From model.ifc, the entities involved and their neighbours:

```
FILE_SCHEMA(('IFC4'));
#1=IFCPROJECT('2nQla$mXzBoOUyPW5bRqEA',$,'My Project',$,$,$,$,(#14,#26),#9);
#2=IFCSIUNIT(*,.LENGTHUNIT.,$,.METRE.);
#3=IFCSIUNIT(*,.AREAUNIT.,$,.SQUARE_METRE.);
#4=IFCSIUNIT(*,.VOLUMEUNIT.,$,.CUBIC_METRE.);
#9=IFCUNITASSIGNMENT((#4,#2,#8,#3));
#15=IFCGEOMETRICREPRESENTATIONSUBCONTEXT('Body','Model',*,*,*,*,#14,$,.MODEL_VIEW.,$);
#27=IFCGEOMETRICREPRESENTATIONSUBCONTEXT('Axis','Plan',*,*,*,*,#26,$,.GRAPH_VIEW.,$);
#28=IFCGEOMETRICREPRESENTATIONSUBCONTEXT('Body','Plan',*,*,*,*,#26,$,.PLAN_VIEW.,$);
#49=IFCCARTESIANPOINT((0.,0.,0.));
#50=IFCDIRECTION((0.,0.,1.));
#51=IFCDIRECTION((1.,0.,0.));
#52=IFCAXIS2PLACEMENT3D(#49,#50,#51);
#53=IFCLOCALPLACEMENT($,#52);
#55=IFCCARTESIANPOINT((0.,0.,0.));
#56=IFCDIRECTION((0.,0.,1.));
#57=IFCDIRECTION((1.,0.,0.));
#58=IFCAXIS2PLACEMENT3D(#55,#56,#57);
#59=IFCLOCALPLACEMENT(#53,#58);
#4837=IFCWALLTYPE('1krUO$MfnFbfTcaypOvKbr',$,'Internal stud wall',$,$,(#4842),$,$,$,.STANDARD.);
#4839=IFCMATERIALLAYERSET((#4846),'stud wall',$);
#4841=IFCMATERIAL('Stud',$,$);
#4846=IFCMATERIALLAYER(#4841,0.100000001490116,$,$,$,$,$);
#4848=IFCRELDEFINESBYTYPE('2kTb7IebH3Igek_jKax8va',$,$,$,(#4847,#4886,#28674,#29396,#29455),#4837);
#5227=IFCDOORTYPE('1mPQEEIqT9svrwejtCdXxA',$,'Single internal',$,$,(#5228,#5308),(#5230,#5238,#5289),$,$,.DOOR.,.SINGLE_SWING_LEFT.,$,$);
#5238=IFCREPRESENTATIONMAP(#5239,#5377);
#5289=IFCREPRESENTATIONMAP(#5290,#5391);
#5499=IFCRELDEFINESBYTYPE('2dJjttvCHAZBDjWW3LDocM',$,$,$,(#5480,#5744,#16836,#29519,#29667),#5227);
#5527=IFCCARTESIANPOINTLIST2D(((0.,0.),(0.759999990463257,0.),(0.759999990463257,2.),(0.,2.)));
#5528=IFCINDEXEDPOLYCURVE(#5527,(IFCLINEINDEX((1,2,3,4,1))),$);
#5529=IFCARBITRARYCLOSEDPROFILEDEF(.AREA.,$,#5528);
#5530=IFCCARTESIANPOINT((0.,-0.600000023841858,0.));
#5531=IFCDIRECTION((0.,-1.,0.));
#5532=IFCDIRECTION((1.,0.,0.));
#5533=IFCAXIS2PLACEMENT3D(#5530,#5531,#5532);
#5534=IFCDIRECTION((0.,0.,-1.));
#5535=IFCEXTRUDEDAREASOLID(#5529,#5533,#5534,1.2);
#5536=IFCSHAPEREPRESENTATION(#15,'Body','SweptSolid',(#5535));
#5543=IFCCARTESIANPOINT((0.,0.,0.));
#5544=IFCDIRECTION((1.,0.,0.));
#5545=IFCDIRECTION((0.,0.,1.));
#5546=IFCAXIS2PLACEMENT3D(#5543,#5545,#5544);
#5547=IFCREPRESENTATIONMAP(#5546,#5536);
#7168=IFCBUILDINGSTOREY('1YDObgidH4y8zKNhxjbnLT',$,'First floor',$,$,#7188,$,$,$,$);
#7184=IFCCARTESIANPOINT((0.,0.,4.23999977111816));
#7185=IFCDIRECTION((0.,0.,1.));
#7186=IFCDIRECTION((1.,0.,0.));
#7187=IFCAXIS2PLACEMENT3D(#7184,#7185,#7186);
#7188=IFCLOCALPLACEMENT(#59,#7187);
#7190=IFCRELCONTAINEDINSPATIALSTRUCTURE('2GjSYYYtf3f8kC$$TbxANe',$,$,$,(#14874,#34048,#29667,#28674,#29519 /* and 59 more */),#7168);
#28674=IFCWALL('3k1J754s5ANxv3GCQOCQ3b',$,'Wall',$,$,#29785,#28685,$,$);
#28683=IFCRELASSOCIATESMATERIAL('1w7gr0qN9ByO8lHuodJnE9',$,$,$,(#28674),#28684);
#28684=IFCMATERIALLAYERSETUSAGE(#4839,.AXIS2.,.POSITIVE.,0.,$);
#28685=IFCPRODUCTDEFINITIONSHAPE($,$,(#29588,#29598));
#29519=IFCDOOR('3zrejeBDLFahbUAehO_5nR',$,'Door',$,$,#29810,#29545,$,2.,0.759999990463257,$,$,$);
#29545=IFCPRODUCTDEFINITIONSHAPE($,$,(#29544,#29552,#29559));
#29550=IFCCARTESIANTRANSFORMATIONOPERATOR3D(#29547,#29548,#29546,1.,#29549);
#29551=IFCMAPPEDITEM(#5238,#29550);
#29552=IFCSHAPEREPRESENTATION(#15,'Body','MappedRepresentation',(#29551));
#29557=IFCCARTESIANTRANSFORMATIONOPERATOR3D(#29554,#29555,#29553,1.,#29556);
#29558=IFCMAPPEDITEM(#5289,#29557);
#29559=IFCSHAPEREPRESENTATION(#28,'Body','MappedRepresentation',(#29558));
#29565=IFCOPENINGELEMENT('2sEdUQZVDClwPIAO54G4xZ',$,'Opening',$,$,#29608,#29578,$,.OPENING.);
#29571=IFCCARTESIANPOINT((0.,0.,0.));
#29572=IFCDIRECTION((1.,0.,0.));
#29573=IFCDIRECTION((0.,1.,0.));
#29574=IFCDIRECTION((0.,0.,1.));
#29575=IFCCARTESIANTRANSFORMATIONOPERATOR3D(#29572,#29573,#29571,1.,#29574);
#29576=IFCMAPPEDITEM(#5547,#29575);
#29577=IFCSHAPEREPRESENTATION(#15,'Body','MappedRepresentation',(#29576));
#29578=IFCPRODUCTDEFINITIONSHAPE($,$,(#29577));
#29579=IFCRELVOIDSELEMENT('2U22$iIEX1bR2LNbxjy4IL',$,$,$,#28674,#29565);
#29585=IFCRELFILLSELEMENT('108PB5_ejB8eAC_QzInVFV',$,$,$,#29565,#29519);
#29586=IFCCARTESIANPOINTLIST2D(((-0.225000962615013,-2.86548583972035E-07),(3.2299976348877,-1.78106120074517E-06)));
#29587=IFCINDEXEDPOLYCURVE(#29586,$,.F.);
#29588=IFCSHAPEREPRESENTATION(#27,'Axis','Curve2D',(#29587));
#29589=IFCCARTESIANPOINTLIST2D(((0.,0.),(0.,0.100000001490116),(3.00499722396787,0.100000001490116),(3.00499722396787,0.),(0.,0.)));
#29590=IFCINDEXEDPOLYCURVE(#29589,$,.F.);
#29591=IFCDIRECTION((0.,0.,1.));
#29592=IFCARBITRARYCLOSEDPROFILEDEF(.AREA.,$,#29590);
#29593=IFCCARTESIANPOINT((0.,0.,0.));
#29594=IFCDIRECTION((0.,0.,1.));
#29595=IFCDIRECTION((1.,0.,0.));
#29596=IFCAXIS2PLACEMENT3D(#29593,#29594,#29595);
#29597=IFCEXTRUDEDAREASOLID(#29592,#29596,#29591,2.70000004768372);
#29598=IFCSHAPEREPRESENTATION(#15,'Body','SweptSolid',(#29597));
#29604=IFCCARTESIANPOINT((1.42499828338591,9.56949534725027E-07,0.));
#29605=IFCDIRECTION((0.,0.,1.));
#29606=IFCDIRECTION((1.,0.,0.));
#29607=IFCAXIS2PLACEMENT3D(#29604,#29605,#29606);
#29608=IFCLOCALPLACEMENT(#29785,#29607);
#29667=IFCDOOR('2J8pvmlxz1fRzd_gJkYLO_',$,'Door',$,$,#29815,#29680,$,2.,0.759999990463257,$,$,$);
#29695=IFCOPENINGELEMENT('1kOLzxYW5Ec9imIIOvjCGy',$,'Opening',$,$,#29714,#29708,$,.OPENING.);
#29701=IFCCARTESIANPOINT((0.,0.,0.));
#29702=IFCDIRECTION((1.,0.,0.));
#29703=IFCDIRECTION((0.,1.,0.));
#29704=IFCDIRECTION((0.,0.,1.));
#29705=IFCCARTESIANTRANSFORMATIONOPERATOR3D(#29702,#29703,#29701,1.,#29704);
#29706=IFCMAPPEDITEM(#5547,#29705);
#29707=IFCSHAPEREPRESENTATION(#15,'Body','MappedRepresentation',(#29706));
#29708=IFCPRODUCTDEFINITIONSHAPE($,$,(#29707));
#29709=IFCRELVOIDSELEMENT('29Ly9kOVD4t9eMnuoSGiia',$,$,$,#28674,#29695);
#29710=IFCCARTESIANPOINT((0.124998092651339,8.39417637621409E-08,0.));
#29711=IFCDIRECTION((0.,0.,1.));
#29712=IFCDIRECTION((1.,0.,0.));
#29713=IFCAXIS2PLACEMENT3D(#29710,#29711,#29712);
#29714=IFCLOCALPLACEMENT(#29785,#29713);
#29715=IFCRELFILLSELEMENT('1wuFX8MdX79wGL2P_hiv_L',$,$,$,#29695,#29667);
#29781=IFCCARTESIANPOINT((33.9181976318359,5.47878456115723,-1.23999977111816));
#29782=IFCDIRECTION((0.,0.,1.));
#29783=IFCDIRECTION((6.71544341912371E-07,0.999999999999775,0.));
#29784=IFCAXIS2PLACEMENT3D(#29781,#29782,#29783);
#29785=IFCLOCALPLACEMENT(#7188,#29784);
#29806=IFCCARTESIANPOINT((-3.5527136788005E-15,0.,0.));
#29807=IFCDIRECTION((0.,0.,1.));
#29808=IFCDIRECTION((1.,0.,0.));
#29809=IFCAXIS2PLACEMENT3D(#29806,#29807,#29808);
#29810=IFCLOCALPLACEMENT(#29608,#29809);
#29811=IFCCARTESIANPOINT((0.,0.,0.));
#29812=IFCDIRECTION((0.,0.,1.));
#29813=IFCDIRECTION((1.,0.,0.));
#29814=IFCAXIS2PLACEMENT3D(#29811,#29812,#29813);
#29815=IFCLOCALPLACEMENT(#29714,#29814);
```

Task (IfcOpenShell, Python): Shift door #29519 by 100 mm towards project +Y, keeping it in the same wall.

```python
import ifcopenshell
import ifcopenshell.api.geometry
import ifcopenshell.util.placement
import ifcopenshell.util.unit

model = ifcopenshell.open("model.ifc")
unit_scale = ifcopenshell.util.unit.calculate_unit_scale(model)

door = model.by_id(29519)
opening = door.FillsVoids[0].RelatingOpeningElement
wall = opening.VoidsElements[0].RelatingBuildingElement

wall_matrix = ifcopenshell.util.placement.get_local_placement(wall.ObjectPlacement)
shift = wall_matrix[:3, 0] * 0.1 / unit_scale
before = ifcopenshell.util.placement.get_local_placement(door.ObjectPlacement)[:3, 3].copy()

# The door is placed relative to its opening, so it follows when the opening moves.
matrix = ifcopenshell.util.placement.get_local_placement(opening.ObjectPlacement)
matrix[:3, 3] += shift
ifcopenshell.api.geometry.edit_object_placement(
    model, product=opening, matrix=matrix, is_si=False, should_transform_children=True
)

after = ifcopenshell.util.placement.get_local_placement(door.ObjectPlacement)[:3, 3]
print("door moved by", (after - before).round(3) + 0.0)

model.write("model_edited.ifc")
```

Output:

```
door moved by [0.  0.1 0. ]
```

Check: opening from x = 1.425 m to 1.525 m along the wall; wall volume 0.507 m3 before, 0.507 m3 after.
